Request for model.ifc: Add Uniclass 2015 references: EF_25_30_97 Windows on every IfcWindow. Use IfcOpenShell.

First a look at what the model holds.

```python
import ifcopenshell

model = ifcopenshell.open("model.ifc")
print(model.schema)
print("classifications:", [c.Name for c in model.by_type("IfcClassification")])
for ifc_class in ("IfcDoor", "IfcRoof", "IfcStair", "IfcWall", "IfcWindow"):
    print(ifc_class, len(model.by_type(ifc_class)))
```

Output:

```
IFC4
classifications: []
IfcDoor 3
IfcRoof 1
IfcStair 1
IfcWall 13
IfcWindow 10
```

```python
import ifcopenshell
import ifcopenshell.api.classification

model = ifcopenshell.open("model.ifc")

system = ifcopenshell.api.classification.add_classification(model, classification="Uniclass 2015")

codes = {
    "IfcWindow": ("EF_25_30_97", "Windows"),
}
for ifc_class, (code, name) in codes.items():
    products = model.by_type(ifc_class)
    ifcopenshell.api.classification.add_reference(
        model, products=products, classification=system, identification=code, name=name
    )
    print(code, len(products))

model.write("model_v2.ifc")
```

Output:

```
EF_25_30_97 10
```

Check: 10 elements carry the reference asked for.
